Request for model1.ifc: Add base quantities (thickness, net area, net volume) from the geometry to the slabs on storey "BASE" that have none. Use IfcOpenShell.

First a look at what the model holds.

```python
import ifcopenshell
import ifcopenshell.util.element
import ifcopenshell.util.unit

model = ifcopenshell.open("model1.ifc")
print(model.schema)
for unit_type in ("LENGTHUNIT", "AREAUNIT", "VOLUMEUNIT"):
    print(unit_type, ifcopenshell.util.unit.calculate_unit_scale(model, unit_type))
storey = next(s for s in model.by_type("IfcBuildingStorey") if s.Name == "BASE")
slabs = [e for e in ifcopenshell.util.element.get_decomposition(storey) if e.is_a("IfcSlab")]
for e in sorted(slabs, key=lambda e: e.id()):
    print(e.id(), e.is_a(), e.Name, list(ifcopenshell.util.element.get_psets(e, qtos_only=True)), sep=" | ")
```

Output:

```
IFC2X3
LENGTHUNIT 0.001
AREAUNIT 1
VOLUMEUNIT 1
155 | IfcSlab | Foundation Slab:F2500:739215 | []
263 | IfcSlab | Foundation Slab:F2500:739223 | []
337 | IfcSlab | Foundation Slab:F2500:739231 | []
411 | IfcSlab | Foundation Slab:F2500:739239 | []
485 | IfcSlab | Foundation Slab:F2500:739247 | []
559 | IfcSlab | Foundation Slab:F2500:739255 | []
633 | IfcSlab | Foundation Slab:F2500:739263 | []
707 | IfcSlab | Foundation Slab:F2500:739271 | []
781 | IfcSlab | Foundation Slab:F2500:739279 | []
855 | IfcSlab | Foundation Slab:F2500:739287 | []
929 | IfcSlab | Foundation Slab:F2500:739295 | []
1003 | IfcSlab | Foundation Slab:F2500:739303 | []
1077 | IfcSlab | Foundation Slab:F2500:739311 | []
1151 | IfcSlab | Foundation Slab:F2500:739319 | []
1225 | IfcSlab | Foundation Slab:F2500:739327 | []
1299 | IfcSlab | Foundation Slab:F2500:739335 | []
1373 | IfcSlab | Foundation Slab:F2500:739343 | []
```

```python
import ifcopenshell
import ifcopenshell.api.pset
import ifcopenshell.geom
import ifcopenshell.util.element
import ifcopenshell.util.shape
import ifcopenshell.util.unit

model = ifcopenshell.open("model1.ifc")
unit_scale = ifcopenshell.util.unit.calculate_unit_scale(model)
area_scale = ifcopenshell.util.unit.calculate_unit_scale(model, "AREAUNIT")
volume_scale = ifcopenshell.util.unit.calculate_unit_scale(model, "VOLUMEUNIT")
settings = ifcopenshell.geom.settings()

storey = next(s for s in model.by_type("IfcBuildingStorey") if s.Name == "BASE")
slabs = [e for e in ifcopenshell.util.element.get_decomposition(storey) if e.is_a("IfcSlab")]

for e in sorted(slabs, key=lambda e: e.id()):
    if ifcopenshell.util.element.get_psets(e, qtos_only=True, should_inherit=False):
        continue
    # Geometry comes back in metres, in the element's own axes.
    shape = ifcopenshell.geom.create_shape(settings, e)
    values = {
        "Width": ifcopenshell.util.shape.get_z(shape.geometry) / unit_scale,
        "NetArea": ifcopenshell.util.shape.get_footprint_area(shape.geometry) / area_scale,
        "NetVolume": ifcopenshell.util.shape.get_volume(shape.geometry) / volume_scale,
    }
    qto = ifcopenshell.api.pset.add_qto(model, product=e, name="BaseQuantities")
    ifcopenshell.api.pset.edit_qto(model, qto=qto, properties=values)
    print(e.id(), {k: round(v, 3) for k, v in values.items()})

model.write("model1_updated.ifc")
```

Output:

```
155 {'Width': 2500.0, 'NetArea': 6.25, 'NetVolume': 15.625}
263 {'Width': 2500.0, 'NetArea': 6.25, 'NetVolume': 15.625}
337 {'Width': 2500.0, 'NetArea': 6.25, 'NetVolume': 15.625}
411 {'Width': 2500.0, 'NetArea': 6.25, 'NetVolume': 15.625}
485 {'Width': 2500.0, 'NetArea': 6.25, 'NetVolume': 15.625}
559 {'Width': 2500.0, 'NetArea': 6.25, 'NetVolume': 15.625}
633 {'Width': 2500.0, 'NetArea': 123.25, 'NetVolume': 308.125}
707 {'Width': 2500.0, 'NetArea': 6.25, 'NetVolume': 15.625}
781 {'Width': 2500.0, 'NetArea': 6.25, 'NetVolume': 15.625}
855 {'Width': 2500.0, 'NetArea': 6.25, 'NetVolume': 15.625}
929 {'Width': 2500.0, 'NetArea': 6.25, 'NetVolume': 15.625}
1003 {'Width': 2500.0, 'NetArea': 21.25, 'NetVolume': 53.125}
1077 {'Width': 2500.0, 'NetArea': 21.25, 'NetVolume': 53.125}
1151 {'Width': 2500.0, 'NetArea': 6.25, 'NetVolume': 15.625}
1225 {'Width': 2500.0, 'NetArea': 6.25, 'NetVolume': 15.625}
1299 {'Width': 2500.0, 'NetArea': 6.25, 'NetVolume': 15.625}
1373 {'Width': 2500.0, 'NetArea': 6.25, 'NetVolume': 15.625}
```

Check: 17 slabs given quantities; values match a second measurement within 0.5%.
